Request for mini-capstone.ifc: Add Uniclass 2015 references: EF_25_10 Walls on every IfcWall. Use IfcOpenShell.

First a look at what the model holds.

```python
import ifcopenshell

model = ifcopenshell.open("mini-capstone.ifc")
print(model.schema)
print("classifications:", [c.Name for c in model.by_type("IfcClassification")])
for ifc_class in ("IfcDoor", "IfcRoof", "IfcStair", "IfcWall", "IfcWindow"):
    print(ifc_class, len(model.by_type(ifc_class)))
```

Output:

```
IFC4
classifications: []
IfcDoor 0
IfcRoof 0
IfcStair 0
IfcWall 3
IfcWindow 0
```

```python
import ifcopenshell
import ifcopenshell.api.classification

model = ifcopenshell.open("mini-capstone.ifc")

system = ifcopenshell.api.classification.add_classification(model, classification="Uniclass 2015")

codes = {
    "IfcWall": ("EF_25_10", "Walls"),
}
for ifc_class, (code, name) in codes.items():
    products = model.by_type(ifc_class)
    ifcopenshell.api.classification.add_reference(
        model, products=products, classification=system, identification=code, name=name
    )
    print(code, len(products))

model.write("mini-capstone_rev.ifc")
```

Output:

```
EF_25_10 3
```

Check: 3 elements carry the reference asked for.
